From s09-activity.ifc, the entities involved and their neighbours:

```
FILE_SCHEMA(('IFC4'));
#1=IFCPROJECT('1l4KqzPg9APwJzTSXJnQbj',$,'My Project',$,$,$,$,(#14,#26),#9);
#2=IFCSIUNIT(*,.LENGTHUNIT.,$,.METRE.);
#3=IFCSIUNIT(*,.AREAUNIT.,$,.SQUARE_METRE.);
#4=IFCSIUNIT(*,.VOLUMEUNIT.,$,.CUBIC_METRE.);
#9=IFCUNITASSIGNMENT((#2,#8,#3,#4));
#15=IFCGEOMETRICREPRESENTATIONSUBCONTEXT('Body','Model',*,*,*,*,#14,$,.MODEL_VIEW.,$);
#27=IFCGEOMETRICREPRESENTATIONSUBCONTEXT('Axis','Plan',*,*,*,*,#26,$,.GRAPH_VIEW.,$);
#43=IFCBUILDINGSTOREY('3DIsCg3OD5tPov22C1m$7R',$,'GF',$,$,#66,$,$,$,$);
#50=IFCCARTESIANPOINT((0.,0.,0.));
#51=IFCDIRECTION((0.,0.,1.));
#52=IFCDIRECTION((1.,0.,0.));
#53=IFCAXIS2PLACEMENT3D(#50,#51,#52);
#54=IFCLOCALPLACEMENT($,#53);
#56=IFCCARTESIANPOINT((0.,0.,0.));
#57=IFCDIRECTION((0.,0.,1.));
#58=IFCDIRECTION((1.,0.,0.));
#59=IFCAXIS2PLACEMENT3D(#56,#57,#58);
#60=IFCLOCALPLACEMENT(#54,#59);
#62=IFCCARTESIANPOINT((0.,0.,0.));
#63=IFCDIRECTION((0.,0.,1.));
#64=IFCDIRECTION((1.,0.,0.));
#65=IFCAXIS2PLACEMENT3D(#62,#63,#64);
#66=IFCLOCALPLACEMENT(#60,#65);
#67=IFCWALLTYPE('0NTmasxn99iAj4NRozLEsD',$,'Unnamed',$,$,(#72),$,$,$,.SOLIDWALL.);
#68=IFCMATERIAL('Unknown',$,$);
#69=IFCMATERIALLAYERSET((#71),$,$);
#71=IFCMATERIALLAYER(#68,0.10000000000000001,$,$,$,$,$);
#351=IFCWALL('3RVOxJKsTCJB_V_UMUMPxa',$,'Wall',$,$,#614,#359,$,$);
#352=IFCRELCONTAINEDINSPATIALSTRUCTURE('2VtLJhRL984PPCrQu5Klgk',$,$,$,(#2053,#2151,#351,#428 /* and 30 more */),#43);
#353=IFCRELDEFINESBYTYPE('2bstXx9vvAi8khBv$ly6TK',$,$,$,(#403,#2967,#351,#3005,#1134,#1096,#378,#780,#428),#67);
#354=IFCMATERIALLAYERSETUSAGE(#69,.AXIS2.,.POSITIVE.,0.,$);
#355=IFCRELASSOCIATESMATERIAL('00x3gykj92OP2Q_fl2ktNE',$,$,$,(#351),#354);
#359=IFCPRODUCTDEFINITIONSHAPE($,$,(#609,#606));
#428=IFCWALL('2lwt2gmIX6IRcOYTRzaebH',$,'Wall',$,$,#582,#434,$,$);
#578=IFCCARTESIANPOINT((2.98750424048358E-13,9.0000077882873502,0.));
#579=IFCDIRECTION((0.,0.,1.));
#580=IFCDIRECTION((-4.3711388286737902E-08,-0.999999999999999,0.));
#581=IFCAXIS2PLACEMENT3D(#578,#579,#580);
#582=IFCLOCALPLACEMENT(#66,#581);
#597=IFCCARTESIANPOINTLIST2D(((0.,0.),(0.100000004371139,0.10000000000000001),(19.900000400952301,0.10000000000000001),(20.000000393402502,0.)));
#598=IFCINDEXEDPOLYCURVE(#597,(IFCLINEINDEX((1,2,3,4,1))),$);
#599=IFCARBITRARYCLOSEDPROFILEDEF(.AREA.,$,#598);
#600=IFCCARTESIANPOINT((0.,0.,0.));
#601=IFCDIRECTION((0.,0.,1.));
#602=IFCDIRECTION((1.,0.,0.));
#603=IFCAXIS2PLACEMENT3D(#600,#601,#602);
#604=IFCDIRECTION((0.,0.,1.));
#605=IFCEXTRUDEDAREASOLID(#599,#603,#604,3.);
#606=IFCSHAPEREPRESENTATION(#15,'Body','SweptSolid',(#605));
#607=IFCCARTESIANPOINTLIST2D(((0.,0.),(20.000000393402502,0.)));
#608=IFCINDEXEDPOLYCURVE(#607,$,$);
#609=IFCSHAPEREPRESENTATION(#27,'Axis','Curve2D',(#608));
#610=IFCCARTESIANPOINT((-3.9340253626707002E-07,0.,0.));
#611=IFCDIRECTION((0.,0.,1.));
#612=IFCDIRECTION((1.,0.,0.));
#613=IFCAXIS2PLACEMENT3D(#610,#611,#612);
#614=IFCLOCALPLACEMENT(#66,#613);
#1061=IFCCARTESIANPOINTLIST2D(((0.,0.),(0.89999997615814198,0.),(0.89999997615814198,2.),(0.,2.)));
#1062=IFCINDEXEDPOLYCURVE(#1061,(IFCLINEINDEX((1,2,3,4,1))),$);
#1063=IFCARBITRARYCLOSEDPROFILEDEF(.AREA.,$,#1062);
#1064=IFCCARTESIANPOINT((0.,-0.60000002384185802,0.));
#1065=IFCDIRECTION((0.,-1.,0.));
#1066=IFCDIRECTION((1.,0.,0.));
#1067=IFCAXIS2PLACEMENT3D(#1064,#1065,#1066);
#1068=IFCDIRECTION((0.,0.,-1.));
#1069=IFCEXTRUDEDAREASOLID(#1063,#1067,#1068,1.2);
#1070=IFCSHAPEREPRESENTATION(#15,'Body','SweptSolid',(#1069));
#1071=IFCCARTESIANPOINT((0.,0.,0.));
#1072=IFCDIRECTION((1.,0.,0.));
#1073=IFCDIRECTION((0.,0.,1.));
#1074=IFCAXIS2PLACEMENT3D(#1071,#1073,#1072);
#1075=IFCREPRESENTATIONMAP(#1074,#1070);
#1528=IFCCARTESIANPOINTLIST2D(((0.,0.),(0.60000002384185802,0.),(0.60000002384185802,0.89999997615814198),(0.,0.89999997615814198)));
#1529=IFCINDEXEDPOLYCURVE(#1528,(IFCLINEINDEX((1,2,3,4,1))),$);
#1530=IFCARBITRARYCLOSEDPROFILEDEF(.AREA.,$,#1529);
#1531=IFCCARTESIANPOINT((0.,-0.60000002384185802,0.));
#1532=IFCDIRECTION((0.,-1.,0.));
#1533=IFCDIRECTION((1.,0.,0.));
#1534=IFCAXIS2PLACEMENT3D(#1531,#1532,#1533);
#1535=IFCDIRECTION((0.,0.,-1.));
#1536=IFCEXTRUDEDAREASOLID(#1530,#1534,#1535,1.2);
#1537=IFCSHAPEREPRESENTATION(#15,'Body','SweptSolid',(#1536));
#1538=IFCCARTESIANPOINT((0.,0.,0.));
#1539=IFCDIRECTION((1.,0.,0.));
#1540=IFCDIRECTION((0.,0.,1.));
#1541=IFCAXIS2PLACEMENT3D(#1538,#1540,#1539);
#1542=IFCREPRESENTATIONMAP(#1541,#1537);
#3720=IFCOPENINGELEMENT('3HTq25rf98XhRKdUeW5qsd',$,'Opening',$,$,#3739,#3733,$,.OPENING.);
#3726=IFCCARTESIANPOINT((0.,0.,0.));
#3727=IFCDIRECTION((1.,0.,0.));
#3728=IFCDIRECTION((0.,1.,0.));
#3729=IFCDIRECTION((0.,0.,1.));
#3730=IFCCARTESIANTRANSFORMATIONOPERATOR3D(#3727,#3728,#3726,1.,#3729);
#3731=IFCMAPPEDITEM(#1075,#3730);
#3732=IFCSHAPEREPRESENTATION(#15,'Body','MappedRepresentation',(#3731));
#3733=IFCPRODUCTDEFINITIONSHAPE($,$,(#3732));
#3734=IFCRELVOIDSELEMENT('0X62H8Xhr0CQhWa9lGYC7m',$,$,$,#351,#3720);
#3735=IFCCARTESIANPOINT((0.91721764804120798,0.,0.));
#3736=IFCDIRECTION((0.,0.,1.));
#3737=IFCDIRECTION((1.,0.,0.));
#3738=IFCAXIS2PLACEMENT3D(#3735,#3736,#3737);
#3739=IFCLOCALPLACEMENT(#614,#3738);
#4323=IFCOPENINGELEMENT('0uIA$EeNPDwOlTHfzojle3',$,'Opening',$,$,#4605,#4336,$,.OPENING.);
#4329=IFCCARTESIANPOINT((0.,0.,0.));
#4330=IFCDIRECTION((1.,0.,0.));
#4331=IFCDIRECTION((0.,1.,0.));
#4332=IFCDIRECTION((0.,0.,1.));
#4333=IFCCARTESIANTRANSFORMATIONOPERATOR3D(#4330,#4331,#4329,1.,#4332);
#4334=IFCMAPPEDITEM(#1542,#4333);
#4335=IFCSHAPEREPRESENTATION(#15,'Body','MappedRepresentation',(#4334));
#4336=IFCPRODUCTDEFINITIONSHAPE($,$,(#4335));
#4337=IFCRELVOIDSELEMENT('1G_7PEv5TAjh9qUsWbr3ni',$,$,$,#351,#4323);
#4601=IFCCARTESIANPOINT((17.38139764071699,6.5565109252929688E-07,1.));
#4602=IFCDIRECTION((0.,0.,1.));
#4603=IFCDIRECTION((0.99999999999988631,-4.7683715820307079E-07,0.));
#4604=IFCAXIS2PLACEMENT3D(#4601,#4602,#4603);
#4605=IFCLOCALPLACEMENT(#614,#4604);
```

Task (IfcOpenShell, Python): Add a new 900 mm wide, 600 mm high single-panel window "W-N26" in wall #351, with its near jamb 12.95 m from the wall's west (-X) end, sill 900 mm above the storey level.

```python
import numpy as np
import ifcopenshell
import ifcopenshell.api.feature
import ifcopenshell.api.geometry
import ifcopenshell.api.root
import ifcopenshell.api.spatial
import ifcopenshell.geom
import ifcopenshell.util.element
import ifcopenshell.util.placement
import ifcopenshell.util.representation
import ifcopenshell.util.shape
import ifcopenshell.util.unit

model = ifcopenshell.open("s09-activity.ifc")
unit_scale = ifcopenshell.util.unit.calculate_unit_scale(model)
settings = ifcopenshell.geom.settings()


def volume(element):
    """Net volume in cubic metres, openings subtracted."""
    shape = ifcopenshell.geom.create_shape(settings, element)
    return ifcopenshell.util.shape.get_volume(shape.geometry)


wall = model.by_guid("3RVOxJKsTCJB_V_UMUMPxa")
storey = ifcopenshell.util.element.get_container(wall, ifc_class="IfcBuildingStorey")
context = ifcopenshell.util.representation.get_context(model, "Model", "Body", "MODEL_VIEW")
before = volume(wall)

width, height, from_end, sill = 0.9, 0.6, 12.95, 0.9  # metres

# The wall runs along its own X axis, and the end named is its -X end.
wall_shape = ifcopenshell.geom.create_shape(settings, wall)
x, y, z = ifcopenshell.util.shape.get_vertices(wall_shape.geometry).T
start = x.min() + from_end
face, thickness = float(y.min()), float(y.max() - y.min())
wall_matrix = ifcopenshell.util.placement.get_local_placement(wall.ObjectPlacement)
level = ifcopenshell.util.placement.get_local_placement(storey.ObjectPlacement)[2, 3]


def in_wall(x, y):
    """Placement at x, y metres in the wall's axes, at sill height."""
    matrix = wall_matrix.copy()
    matrix[:, 3] = wall_matrix @ np.array([x / unit_scale, y / unit_scale, 0.0, 1.0])
    matrix[2, 3] = level + sill / unit_scale
    return matrix


# Opening: a box that overshoots both wall faces by 50 mm.
opening = ifcopenshell.api.root.create_entity(model, ifc_class="IfcOpeningElement", predefined_type="OPENING")
box = ifcopenshell.api.geometry.add_wall_representation(
    model, context=context, length=width, height=height, thickness=thickness + 0.1
)
ifcopenshell.api.geometry.assign_representation(model, product=opening, representation=box)
ifcopenshell.api.geometry.edit_object_placement(model, product=opening, matrix=in_wall(start, face - 0.05), is_si=False)
ifcopenshell.api.feature.add_feature(model, feature=opening, element=wall)

window = ifcopenshell.api.root.create_entity(model, ifc_class="IfcWindow", name="W-N26", predefined_type="WINDOW")
window.OverallWidth, window.OverallHeight = width / unit_scale, height / unit_scale
window.PartitioningType = "SINGLE_PANEL"
body = ifcopenshell.api.geometry.add_window_representation(
    model,
    context=context,
    overall_width=window.OverallWidth,
    overall_height=window.OverallHeight,
    partition_type="SINGLE_PANEL",
)
ifcopenshell.api.geometry.assign_representation(model, product=window, representation=body)
ifcopenshell.api.spatial.assign_container(model, products=[window], relating_structure=storey)
ifcopenshell.api.feature.add_filling(model, opening=opening, element=window)

# Centre the window in the wall's thickness.
ifcopenshell.api.geometry.edit_object_placement(model, product=window, matrix=in_wall(start, face), is_si=False)
window_shape = ifcopenshell.geom.create_shape(settings, window)
depth = ifcopenshell.util.shape.get_vertices(window_shape.geometry)[:, 1]
offset = face + thickness / 2 - (depth.min() + depth.max()) / 2
ifcopenshell.api.geometry.edit_object_placement(model, product=window, matrix=in_wall(start, offset), is_si=False)

after = volume(wall)

print(f"wall volume {before:.3f} -> {after:.3f} m3")

model.write("s09-activity_updated.ifc")
```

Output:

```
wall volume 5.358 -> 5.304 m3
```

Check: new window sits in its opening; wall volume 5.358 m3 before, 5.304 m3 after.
